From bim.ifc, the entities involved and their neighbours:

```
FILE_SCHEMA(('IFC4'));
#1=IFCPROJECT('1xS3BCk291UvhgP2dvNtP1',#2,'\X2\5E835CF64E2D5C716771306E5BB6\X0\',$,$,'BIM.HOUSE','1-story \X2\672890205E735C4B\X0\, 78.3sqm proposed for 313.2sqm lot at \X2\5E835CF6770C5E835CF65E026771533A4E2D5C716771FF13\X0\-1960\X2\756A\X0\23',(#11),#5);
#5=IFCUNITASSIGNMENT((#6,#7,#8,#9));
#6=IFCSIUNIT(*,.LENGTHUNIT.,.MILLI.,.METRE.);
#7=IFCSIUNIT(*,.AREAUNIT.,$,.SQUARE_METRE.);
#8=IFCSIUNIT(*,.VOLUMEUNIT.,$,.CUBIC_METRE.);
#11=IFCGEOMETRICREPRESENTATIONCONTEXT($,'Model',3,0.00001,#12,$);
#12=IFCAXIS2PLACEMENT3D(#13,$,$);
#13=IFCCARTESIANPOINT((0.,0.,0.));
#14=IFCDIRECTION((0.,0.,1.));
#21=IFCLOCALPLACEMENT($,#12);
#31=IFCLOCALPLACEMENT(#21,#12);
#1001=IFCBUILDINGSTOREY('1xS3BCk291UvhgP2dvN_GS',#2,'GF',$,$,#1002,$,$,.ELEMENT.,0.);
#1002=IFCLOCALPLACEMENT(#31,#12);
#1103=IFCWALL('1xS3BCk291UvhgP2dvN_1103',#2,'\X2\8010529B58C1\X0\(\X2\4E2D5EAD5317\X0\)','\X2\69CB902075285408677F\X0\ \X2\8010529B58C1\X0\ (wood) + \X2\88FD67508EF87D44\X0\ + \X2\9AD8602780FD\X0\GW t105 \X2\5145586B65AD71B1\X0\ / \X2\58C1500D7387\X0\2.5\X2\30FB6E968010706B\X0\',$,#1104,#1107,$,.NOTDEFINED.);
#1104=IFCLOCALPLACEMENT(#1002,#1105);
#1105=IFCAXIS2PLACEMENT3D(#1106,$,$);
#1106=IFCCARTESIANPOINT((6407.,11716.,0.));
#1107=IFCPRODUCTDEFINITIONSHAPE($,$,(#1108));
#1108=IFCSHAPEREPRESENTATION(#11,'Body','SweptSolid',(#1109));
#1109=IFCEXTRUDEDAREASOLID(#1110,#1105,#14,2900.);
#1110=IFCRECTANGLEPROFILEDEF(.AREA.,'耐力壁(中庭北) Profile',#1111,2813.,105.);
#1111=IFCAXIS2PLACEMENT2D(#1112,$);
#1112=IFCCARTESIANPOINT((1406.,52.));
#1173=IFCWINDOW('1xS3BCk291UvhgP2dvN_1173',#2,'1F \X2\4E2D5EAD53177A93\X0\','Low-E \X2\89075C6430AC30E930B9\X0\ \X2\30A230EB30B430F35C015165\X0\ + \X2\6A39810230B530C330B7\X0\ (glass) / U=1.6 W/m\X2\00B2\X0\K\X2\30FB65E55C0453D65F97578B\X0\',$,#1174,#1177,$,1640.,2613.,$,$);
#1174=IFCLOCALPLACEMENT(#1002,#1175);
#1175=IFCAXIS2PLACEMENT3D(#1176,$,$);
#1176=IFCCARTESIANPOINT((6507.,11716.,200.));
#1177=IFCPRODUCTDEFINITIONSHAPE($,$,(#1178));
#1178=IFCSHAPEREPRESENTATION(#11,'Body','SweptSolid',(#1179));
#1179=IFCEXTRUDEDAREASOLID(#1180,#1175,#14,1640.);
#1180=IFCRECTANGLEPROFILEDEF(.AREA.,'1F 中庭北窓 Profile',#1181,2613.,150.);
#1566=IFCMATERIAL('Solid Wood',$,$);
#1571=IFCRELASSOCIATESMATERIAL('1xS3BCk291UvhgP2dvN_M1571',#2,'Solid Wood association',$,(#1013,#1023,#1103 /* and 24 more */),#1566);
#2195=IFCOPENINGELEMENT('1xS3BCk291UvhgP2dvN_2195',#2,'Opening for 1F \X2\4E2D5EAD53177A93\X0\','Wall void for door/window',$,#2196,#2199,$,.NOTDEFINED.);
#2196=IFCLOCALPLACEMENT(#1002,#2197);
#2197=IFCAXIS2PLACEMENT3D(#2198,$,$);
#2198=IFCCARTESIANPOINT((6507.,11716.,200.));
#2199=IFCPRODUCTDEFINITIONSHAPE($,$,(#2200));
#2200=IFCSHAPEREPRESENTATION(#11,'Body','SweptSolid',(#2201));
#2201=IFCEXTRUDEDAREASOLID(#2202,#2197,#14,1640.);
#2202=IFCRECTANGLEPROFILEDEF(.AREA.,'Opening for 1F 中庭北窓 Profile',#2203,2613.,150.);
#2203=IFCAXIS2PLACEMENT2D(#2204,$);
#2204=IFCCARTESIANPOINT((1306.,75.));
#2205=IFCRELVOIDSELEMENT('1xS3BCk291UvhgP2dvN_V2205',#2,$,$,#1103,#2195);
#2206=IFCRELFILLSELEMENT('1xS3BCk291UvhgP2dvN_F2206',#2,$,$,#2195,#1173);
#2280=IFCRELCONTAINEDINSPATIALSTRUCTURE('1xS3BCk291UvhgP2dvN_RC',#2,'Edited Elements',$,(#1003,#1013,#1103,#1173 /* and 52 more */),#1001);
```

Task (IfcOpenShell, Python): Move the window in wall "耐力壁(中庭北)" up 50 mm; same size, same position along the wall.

```python
import numpy as np
import ifcopenshell
import ifcopenshell.api.geometry
import ifcopenshell.util.placement
import ifcopenshell.util.unit

model = ifcopenshell.open("bim.ifc")
unit_scale = ifcopenshell.util.unit.calculate_unit_scale(model)

window = model.by_id(1173)
opening = window.FillsVoids[0].RelatingOpeningElement
dz = 0.05 / unit_scale

shift = np.array([0.0, 0.0, dz])
# The window is not placed relative to its opening, so move both.
for product in (opening, window):
    matrix = ifcopenshell.util.placement.get_local_placement(product.ObjectPlacement)
    matrix[:3, 3] += shift
    ifcopenshell.api.geometry.edit_object_placement(model, product=product, matrix=matrix, is_si=False)

print(f"moved by {dz * unit_scale:+.3f} m")

model.write("bim-out.ifc")
```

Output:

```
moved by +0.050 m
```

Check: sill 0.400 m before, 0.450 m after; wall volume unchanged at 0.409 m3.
